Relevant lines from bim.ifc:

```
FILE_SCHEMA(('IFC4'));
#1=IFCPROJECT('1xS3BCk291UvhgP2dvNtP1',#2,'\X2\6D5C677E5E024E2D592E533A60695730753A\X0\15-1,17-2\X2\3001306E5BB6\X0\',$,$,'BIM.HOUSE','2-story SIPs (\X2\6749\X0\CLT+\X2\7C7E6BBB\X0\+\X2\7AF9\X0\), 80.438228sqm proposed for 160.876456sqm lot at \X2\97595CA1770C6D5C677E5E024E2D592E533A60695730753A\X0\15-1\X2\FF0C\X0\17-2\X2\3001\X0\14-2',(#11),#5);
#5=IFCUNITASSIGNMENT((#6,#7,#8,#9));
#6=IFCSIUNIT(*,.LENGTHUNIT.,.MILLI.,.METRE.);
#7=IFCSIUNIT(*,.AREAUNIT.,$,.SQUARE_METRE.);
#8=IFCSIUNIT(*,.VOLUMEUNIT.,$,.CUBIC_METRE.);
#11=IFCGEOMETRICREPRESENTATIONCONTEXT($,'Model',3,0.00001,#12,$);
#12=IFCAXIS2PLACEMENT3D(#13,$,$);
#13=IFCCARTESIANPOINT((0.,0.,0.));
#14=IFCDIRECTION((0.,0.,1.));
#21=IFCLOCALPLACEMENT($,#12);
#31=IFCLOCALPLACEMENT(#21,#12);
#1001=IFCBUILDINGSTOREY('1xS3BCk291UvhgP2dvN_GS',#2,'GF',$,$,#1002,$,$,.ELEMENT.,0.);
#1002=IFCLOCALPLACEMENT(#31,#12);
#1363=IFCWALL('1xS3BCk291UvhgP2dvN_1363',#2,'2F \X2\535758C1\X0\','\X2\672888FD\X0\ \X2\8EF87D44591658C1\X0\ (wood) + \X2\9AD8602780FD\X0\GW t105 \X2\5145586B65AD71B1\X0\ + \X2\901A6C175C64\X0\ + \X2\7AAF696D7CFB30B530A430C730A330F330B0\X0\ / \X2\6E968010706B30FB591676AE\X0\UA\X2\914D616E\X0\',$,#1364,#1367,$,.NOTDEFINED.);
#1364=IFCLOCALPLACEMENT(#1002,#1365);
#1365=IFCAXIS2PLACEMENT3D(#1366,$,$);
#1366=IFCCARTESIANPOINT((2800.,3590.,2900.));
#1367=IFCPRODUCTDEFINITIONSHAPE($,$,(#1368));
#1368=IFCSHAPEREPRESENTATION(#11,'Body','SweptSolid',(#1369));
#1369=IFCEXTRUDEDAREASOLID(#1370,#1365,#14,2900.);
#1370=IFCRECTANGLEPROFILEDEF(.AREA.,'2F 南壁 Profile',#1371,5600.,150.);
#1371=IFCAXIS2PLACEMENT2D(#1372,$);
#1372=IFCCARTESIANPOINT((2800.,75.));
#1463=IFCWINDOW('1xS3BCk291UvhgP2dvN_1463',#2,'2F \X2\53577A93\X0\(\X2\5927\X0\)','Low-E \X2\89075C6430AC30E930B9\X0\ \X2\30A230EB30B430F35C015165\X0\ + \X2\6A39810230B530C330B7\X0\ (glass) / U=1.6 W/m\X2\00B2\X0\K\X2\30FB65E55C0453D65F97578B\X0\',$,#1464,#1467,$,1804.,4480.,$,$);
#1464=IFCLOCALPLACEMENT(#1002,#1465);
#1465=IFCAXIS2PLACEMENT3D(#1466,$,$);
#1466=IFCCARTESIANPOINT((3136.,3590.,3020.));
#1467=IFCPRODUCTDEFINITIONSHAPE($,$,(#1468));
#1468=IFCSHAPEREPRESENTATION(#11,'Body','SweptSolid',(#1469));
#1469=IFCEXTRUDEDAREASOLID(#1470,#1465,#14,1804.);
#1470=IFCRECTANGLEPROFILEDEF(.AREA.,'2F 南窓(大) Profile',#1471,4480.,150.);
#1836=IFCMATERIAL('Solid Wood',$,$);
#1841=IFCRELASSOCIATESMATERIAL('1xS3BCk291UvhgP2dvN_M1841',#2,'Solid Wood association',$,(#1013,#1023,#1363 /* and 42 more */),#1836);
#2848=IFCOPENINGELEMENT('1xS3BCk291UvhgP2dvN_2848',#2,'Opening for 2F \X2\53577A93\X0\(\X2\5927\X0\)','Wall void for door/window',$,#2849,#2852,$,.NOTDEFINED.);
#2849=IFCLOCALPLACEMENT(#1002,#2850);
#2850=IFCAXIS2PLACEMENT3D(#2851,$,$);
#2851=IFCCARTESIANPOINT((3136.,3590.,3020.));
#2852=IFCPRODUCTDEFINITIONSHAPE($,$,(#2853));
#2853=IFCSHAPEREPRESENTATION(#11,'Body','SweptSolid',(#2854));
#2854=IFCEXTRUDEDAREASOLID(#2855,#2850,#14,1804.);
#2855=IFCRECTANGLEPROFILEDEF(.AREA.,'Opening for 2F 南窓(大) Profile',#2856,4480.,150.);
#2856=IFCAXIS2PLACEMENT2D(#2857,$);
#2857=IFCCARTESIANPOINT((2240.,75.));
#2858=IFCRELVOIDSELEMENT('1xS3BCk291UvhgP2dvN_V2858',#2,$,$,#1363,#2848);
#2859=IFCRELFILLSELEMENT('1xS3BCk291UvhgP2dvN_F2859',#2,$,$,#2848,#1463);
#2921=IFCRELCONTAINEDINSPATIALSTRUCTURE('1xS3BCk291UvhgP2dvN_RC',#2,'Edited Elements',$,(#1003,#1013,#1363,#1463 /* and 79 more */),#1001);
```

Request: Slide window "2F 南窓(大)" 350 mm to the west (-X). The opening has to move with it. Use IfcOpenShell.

```python
import ifcopenshell
import ifcopenshell.api.geometry
import ifcopenshell.util.placement
import ifcopenshell.util.unit

model = ifcopenshell.open("bim.ifc")
unit_scale = ifcopenshell.util.unit.calculate_unit_scale(model)

window = model.by_guid("1xS3BCk291UvhgP2dvN_1463")
opening = window.FillsVoids[0].RelatingOpeningElement
wall = opening.VoidsElements[0].RelatingBuildingElement

wall_matrix = ifcopenshell.util.placement.get_local_placement(wall.ObjectPlacement)
shift = wall_matrix[:3, 0] * -0.35 / unit_scale
before = ifcopenshell.util.placement.get_local_placement(window.ObjectPlacement)[:3, 3].copy()

# The window is not placed relative to its opening, so move both.
for product in (opening, window):
    matrix = ifcopenshell.util.placement.get_local_placement(product.ObjectPlacement)
    matrix[:3, 3] += shift
    ifcopenshell.api.geometry.edit_object_placement(model, product=product, matrix=matrix, is_si=False)

after = ifcopenshell.util.placement.get_local_placement(window.ObjectPlacement)[:3, 3]
print("window moved by", (after - before).round(3) + 0.0)

model.write("bim_rev.ifc")
```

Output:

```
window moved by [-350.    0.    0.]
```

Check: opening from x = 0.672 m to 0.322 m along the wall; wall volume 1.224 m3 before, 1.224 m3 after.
